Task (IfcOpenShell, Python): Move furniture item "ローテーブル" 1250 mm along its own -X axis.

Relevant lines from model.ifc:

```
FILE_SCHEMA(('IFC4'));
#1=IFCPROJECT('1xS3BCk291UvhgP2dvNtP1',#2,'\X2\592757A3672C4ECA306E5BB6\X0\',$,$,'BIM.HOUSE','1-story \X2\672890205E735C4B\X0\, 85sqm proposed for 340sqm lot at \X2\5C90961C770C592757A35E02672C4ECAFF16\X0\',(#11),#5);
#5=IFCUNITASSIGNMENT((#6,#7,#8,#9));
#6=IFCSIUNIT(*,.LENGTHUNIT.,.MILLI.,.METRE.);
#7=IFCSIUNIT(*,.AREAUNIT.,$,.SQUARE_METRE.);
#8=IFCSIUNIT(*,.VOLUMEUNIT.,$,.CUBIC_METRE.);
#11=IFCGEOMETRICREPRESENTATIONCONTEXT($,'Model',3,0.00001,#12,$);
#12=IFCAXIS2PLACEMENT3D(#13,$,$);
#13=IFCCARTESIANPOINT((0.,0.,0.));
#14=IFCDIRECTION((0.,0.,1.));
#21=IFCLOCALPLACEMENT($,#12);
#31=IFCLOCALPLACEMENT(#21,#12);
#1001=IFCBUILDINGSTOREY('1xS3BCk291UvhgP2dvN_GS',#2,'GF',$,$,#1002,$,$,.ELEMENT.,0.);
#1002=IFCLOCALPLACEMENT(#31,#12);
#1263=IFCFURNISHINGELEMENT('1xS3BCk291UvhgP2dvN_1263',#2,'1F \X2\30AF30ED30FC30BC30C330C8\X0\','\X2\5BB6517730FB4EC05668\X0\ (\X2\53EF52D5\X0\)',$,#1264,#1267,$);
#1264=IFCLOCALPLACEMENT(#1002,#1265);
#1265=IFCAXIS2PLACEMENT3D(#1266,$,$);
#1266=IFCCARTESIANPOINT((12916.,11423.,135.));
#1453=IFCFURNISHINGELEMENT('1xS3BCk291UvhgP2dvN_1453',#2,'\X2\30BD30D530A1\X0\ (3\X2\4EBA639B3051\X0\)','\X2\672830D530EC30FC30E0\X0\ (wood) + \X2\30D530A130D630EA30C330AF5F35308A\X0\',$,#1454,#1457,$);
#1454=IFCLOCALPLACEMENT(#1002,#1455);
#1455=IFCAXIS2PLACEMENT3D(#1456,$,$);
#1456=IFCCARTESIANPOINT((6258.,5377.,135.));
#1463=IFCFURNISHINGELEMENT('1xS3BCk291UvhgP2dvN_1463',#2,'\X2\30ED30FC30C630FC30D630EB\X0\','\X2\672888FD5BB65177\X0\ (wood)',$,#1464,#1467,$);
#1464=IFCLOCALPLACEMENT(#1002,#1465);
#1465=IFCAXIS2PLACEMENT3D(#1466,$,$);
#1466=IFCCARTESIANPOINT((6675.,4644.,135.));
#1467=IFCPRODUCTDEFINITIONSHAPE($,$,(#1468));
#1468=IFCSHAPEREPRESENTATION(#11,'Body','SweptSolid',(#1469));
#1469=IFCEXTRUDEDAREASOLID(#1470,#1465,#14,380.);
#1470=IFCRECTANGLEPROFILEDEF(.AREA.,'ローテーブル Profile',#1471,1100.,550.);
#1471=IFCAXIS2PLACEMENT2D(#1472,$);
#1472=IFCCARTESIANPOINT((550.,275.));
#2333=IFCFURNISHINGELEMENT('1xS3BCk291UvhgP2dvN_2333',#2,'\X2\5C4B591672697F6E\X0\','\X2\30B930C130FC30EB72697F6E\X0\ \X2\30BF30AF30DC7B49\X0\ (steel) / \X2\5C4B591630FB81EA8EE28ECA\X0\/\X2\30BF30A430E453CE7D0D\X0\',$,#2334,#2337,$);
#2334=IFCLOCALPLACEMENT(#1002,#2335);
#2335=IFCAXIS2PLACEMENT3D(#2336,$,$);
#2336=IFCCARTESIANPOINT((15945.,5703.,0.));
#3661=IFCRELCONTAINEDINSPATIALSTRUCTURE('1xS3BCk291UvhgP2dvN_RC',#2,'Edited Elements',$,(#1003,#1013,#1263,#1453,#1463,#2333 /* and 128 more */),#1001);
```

```python
import ifcopenshell
import ifcopenshell.api.geometry
import ifcopenshell.util.placement

model = ifcopenshell.open("model.ifc")

item = model.by_id(1463)
matrix = ifcopenshell.util.placement.get_local_placement(item.ObjectPlacement)
matrix[:3, 3] -= matrix[:3, 0] * 1250.0
ifcopenshell.api.geometry.edit_object_placement(model, product=item, matrix=matrix, is_si=False)

print(ifcopenshell.util.placement.get_local_placement(item.ObjectPlacement).round(3) + 0.0)

model.write("model_updated.ifc")
```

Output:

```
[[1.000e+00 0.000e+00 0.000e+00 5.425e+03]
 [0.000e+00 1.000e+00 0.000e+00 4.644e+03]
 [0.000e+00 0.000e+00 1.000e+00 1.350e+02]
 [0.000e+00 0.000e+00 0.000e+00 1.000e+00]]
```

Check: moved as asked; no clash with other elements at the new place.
